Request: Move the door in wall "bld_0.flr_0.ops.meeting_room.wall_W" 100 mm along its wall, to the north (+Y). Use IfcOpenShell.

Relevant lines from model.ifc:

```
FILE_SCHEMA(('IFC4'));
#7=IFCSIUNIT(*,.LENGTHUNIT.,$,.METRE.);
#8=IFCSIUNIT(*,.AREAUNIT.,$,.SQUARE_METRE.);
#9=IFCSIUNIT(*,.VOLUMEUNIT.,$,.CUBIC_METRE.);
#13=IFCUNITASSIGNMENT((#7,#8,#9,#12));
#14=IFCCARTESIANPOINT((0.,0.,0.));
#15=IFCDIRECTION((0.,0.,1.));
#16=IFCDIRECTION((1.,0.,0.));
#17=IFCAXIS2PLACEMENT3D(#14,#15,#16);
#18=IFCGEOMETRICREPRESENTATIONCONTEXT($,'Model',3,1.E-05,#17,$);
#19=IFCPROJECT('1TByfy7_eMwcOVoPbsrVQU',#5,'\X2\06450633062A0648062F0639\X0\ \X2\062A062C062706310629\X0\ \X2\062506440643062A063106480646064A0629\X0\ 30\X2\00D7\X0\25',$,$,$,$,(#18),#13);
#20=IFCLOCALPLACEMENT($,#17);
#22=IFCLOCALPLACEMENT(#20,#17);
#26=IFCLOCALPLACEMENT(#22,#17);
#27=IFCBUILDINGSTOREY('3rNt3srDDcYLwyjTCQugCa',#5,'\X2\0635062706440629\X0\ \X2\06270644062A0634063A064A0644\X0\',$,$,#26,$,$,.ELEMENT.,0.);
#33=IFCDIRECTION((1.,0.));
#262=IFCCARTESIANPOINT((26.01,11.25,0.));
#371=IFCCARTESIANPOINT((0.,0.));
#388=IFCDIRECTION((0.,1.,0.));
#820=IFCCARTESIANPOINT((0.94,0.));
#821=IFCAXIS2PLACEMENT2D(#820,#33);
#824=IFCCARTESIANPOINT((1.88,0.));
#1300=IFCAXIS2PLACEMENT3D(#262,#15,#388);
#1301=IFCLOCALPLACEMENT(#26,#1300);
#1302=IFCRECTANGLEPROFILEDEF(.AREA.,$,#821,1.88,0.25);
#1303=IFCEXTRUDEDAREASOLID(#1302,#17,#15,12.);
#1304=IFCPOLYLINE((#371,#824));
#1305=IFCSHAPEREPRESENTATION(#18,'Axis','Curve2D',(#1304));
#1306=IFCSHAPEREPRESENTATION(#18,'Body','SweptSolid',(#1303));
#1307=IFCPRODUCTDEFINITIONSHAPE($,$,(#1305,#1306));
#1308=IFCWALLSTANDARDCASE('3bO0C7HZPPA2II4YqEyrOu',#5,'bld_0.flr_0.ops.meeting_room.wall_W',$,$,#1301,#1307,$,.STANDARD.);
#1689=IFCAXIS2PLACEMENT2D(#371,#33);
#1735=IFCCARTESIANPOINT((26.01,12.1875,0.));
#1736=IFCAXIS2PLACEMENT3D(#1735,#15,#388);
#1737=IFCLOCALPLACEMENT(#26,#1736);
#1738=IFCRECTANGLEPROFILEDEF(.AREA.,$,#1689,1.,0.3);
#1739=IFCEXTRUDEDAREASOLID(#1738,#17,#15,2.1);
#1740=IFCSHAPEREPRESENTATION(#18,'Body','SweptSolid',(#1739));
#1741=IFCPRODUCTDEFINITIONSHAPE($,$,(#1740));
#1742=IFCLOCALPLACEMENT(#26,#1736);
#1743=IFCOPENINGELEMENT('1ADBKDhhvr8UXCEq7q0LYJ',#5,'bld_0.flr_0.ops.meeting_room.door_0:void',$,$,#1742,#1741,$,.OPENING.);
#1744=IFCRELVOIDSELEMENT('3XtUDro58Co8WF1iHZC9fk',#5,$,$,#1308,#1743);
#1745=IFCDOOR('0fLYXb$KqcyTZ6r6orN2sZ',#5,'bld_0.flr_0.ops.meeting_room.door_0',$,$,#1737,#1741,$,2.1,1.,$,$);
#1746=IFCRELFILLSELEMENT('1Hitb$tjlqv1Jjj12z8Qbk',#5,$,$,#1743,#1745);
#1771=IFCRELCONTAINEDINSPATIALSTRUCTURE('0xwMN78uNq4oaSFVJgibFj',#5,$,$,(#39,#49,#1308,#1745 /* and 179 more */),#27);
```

```python
import ifcopenshell
import ifcopenshell.api.geometry
import ifcopenshell.util.placement
import ifcopenshell.util.unit

model = ifcopenshell.open("model.ifc")
unit_scale = ifcopenshell.util.unit.calculate_unit_scale(model)

door = model.by_guid("0fLYXb$KqcyTZ6r6orN2sZ")
opening = door.FillsVoids[0].RelatingOpeningElement
wall = opening.VoidsElements[0].RelatingBuildingElement

wall_matrix = ifcopenshell.util.placement.get_local_placement(wall.ObjectPlacement)
shift = wall_matrix[:3, 0] * 0.1 / unit_scale
before = ifcopenshell.util.placement.get_local_placement(door.ObjectPlacement)[:3, 3].copy()

# The door is not placed relative to its opening, so move both.
for product in (opening, door):
    matrix = ifcopenshell.util.placement.get_local_placement(product.ObjectPlacement)
    matrix[:3, 3] += shift
    ifcopenshell.api.geometry.edit_object_placement(model, product=product, matrix=matrix, is_si=False)

after = ifcopenshell.util.placement.get_local_placement(door.ObjectPlacement)[:3, 3]
print("door moved by", (after - before).round(3) + 0.0)

model.write("model-out.ifc")
```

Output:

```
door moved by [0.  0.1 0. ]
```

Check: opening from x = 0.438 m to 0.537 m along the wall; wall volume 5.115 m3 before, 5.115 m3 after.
